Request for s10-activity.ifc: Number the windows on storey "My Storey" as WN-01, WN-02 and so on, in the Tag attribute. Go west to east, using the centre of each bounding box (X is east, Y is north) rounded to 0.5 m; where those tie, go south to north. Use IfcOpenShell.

First a look at what the model holds.

```python
import ifcopenshell
import ifcopenshell.util.element
import ifcopenshell.util.placement

model = ifcopenshell.open("s10-activity.ifc")
print(model.schema)
storey = next(s for s in model.by_type("IfcBuildingStorey") if s.Name == "My Storey")
windows = [e for e in ifcopenshell.util.element.get_decomposition(storey) if e.is_a("IfcWindow")]
for e in sorted(windows, key=lambda e: e.id()):
    origin = ifcopenshell.util.placement.get_local_placement(e.ObjectPlacement)[:3, 3]
    print(e.id(), e.Tag, e.Name, origin.round(2) + 0.0, sep=" | ")
```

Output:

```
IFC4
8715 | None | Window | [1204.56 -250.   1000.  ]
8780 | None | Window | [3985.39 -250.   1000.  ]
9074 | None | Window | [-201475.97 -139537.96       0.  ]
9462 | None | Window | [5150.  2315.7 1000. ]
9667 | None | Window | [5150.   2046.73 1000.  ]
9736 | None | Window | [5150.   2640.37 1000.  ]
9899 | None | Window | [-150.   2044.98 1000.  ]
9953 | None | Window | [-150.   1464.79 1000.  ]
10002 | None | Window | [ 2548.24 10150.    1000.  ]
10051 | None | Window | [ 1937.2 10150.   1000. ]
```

```python
import ifcopenshell
import ifcopenshell.geom
import ifcopenshell.util.element
import ifcopenshell.util.shape

model = ifcopenshell.open("s10-activity.ifc")
settings = ifcopenshell.geom.settings()
settings.set("use-world-coords", True)


def centre(element):
    shape = ifcopenshell.geom.create_shape(settings, element)
    return ifcopenshell.util.shape.get_bbox_centroid(shape.geometry)


storey = next(s for s in model.by_type("IfcBuildingStorey") if s.Name == "My Storey")
windows = [e for e in ifcopenshell.util.element.get_decomposition(storey) if e.is_a("IfcWindow")]

# Insertion points can sit at a corner or the storey origin, so sort by the geometry (in metres).
centres = {e: centre(e) for e in windows}
windows.sort(key=lambda e: (round(centres[e][0] / 0.5), centres[e][1]))

for i, e in enumerate(windows, start=1):
    number = f"WN-{i:02d}"
    e.Tag = number
    print(e.id(), number)

model.write("s10-activity_rev.ifc")
```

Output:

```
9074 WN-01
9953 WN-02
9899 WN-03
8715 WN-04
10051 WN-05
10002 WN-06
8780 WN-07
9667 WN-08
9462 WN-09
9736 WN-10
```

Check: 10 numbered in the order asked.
